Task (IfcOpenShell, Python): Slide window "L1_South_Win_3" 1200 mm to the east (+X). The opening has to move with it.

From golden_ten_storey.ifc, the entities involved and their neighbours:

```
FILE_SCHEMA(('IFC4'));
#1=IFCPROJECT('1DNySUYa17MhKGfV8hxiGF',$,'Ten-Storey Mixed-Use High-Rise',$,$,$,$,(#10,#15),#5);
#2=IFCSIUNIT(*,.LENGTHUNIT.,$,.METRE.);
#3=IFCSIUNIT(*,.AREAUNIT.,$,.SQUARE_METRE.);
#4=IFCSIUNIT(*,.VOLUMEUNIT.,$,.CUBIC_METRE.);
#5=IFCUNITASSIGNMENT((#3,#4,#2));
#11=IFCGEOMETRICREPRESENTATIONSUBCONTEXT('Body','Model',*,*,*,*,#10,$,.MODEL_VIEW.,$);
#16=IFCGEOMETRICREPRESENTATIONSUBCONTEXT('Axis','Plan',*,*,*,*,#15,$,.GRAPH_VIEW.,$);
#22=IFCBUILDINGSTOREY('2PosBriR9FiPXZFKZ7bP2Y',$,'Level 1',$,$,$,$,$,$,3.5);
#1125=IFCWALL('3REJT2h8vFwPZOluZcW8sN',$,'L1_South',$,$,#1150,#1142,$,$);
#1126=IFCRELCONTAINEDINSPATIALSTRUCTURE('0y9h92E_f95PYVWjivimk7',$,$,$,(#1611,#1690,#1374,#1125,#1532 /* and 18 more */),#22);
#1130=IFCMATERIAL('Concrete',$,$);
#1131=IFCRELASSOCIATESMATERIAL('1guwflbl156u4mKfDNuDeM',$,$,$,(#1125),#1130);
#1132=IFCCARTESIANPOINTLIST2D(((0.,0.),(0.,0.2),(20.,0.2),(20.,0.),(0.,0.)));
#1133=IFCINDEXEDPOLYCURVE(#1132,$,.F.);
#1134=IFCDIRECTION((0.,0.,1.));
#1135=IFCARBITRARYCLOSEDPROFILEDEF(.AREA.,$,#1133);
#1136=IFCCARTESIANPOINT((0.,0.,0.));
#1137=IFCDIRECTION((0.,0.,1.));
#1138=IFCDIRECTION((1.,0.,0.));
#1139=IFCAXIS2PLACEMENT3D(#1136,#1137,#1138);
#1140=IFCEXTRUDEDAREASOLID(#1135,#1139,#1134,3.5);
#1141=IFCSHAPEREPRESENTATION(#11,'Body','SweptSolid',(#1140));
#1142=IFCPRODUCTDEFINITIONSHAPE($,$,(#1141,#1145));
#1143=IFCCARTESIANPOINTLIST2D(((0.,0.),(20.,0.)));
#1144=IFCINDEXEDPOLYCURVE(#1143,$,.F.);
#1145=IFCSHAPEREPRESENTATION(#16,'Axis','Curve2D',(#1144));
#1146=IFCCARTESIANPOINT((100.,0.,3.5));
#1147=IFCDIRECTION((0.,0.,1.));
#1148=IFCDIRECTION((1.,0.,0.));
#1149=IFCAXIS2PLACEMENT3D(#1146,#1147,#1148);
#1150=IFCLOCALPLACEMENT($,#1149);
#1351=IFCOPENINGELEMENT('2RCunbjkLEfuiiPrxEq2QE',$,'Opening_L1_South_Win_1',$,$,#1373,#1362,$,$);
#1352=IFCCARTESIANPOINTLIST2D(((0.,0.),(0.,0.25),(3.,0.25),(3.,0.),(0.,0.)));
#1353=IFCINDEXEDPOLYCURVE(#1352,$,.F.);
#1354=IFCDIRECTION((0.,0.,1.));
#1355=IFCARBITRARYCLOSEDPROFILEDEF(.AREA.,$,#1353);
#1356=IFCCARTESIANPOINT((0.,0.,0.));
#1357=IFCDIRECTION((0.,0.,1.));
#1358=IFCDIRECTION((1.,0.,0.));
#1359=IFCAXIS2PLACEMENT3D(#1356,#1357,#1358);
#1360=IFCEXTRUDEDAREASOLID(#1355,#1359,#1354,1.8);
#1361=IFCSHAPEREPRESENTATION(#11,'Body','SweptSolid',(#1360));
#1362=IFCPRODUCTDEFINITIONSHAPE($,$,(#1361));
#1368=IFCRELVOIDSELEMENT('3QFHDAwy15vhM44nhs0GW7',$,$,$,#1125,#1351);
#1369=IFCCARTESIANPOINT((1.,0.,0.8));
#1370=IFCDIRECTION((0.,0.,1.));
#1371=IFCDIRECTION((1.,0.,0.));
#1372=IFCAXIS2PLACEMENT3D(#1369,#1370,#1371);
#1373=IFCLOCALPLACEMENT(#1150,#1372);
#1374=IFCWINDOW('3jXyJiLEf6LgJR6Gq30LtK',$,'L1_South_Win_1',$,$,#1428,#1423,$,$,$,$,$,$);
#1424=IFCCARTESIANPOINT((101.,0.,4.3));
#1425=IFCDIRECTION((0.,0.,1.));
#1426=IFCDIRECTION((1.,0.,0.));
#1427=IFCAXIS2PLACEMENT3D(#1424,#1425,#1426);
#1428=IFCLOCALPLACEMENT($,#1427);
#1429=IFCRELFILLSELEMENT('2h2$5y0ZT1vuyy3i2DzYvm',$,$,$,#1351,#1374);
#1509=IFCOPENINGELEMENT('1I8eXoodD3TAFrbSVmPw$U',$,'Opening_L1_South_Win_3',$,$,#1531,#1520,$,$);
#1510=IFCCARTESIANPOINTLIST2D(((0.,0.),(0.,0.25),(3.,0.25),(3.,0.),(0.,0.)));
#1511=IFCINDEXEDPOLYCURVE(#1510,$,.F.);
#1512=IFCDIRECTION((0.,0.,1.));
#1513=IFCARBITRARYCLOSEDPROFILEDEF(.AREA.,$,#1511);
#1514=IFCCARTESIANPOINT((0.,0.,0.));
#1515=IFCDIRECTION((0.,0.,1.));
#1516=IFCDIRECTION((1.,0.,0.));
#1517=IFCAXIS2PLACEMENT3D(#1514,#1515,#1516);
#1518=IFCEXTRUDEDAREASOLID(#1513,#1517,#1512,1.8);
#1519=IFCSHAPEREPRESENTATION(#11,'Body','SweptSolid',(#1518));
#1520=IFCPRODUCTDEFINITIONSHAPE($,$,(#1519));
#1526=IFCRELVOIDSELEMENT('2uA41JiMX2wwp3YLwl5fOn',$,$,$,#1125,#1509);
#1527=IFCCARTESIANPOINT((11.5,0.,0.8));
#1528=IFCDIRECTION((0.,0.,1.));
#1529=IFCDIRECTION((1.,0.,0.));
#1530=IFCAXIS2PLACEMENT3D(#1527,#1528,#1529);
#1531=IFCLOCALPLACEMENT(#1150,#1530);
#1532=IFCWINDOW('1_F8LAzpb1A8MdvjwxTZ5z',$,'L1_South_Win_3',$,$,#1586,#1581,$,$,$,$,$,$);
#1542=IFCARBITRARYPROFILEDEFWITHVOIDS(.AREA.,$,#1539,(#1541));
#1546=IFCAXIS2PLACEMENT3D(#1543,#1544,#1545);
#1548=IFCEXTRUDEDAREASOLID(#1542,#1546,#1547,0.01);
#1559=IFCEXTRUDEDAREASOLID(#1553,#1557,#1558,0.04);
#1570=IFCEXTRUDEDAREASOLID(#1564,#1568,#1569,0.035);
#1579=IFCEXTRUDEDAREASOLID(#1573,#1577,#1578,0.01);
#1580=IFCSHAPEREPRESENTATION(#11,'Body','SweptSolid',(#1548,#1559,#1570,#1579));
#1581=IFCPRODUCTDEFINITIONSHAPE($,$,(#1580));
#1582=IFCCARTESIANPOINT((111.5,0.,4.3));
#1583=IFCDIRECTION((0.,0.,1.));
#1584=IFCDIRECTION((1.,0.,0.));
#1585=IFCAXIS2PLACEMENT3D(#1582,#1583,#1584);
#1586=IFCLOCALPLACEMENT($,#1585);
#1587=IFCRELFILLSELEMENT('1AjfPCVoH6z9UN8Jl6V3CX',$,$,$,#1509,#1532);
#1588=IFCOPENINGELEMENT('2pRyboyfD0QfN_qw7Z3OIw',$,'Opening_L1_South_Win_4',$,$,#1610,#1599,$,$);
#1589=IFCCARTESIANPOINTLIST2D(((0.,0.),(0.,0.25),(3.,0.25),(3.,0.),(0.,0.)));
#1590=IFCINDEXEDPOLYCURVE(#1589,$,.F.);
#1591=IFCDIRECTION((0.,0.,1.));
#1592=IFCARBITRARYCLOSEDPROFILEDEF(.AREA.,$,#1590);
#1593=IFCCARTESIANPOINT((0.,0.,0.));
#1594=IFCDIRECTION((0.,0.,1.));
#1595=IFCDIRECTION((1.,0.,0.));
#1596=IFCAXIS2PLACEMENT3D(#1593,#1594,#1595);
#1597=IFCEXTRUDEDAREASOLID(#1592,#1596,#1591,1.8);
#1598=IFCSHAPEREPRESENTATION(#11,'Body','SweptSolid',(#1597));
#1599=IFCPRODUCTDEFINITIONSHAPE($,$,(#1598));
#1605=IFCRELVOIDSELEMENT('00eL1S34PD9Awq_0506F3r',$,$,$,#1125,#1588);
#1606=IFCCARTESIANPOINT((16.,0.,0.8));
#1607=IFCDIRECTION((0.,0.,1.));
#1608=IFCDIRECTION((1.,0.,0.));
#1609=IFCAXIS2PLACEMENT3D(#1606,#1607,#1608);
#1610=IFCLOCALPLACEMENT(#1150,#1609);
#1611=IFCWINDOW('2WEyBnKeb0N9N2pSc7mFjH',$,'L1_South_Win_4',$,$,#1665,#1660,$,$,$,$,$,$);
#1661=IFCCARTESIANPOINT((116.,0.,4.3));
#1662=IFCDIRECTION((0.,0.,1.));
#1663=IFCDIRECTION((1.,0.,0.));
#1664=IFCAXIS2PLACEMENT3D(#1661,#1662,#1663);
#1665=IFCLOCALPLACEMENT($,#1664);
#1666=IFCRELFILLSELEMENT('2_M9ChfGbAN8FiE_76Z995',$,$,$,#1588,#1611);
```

```python
import ifcopenshell
import ifcopenshell.api.geometry
import ifcopenshell.util.placement
import ifcopenshell.util.unit

model = ifcopenshell.open("golden_ten_storey.ifc")
unit_scale = ifcopenshell.util.unit.calculate_unit_scale(model)

window = model.by_guid("1_F8LAzpb1A8MdvjwxTZ5z")
opening = window.FillsVoids[0].RelatingOpeningElement
wall = opening.VoidsElements[0].RelatingBuildingElement

wall_matrix = ifcopenshell.util.placement.get_local_placement(wall.ObjectPlacement)
shift = wall_matrix[:3, 0] * 1.2 / unit_scale
before = ifcopenshell.util.placement.get_local_placement(window.ObjectPlacement)[:3, 3].copy()

# The window is not placed relative to its opening, so move both.
for product in (opening, window):
    matrix = ifcopenshell.util.placement.get_local_placement(product.ObjectPlacement)
    matrix[:3, 3] += shift
    ifcopenshell.api.geometry.edit_object_placement(model, product=product, matrix=matrix, is_si=False)

after = ifcopenshell.util.placement.get_local_placement(window.ObjectPlacement)[:3, 3]
print("window moved by", (after - before).round(3) + 0.0)

model.write("golden_ten_storey_edited.ifc")
```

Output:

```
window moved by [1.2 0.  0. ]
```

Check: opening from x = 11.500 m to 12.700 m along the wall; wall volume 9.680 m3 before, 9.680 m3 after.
